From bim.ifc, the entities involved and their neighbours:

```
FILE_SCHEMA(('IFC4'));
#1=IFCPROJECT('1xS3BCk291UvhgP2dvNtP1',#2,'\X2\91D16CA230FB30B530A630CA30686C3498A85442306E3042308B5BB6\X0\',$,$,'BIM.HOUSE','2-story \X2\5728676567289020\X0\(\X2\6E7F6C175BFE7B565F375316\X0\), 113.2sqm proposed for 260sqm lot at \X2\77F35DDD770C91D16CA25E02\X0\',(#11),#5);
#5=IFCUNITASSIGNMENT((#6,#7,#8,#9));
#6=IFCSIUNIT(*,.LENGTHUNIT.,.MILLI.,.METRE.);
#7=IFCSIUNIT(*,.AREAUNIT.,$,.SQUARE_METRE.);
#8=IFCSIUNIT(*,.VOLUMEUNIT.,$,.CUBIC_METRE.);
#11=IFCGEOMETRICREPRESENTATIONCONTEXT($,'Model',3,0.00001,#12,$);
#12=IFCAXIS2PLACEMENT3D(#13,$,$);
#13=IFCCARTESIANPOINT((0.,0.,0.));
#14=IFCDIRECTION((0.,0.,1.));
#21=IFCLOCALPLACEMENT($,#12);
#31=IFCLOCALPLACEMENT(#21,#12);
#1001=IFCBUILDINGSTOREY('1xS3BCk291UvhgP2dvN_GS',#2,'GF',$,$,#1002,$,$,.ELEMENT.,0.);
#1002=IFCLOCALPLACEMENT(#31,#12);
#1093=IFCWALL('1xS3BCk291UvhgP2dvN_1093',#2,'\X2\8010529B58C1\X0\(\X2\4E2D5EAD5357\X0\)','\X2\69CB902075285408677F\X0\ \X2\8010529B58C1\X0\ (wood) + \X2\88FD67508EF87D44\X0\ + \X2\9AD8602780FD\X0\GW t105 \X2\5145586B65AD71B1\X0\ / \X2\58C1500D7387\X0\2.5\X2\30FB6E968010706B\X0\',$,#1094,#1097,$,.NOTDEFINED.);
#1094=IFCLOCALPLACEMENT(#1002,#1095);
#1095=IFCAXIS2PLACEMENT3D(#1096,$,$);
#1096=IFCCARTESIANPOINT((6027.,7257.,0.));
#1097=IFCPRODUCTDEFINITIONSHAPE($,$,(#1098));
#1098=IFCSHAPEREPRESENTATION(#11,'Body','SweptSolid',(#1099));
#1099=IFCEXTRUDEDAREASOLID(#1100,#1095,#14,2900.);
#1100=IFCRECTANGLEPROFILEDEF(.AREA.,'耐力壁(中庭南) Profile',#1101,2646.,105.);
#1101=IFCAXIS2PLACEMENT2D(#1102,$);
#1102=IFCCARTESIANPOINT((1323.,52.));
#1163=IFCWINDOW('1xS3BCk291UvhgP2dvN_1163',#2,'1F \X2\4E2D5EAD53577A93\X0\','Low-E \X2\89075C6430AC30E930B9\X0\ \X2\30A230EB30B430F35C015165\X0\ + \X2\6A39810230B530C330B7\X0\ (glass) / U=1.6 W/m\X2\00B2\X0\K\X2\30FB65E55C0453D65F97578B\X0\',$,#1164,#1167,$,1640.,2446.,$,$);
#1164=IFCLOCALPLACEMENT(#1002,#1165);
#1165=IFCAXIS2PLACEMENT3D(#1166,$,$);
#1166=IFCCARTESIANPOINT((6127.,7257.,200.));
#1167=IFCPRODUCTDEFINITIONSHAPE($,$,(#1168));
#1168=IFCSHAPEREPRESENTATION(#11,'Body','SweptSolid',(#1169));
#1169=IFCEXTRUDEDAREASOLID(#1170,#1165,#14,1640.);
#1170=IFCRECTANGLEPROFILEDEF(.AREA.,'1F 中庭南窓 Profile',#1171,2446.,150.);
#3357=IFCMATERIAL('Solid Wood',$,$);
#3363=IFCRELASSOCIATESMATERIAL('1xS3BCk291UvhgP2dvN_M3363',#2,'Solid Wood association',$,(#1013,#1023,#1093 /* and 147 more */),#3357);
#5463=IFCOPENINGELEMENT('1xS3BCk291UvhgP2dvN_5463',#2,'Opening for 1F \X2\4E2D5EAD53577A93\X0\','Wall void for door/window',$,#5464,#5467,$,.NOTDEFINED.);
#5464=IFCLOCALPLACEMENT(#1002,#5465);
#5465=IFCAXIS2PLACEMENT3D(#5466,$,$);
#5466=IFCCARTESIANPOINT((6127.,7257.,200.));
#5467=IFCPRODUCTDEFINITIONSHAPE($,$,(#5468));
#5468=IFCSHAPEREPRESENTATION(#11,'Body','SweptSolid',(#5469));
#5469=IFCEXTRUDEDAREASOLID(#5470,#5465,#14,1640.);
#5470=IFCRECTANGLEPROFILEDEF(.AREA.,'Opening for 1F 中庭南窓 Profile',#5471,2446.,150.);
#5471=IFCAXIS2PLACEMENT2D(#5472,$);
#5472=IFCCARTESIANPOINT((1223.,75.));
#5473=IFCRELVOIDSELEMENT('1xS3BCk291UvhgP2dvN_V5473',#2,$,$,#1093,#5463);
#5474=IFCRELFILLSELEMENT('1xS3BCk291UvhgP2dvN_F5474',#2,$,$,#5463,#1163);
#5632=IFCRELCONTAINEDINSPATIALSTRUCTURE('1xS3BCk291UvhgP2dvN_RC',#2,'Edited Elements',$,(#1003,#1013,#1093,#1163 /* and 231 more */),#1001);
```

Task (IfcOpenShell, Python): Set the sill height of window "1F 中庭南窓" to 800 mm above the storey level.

```python
import numpy as np
import ifcopenshell
import ifcopenshell.api.geometry
import ifcopenshell.geom
import ifcopenshell.util.element
import ifcopenshell.util.placement
import ifcopenshell.util.shape
import ifcopenshell.util.unit

model = ifcopenshell.open("bim.ifc")
unit_scale = ifcopenshell.util.unit.calculate_unit_scale(model)

window = model.by_guid("1xS3BCk291UvhgP2dvN_1163")
opening = window.FillsVoids[0].RelatingOpeningElement
storey = ifcopenshell.util.element.get_container(window, ifc_class="IfcBuildingStorey")
level = ifcopenshell.util.placement.get_local_placement(storey.ObjectPlacement)[2, 3]

# The opening's origin need not be at the sill, so measure its lowest point.
shape = ifcopenshell.geom.create_shape(ifcopenshell.geom.settings(), opening)
bottom = ifcopenshell.util.shape.get_shape_bottom_elevation(shape, shape.geometry) / unit_scale
dz = level + 800.0 - bottom

shift = np.array([0.0, 0.0, dz])
# The window is not placed relative to its opening, so move both.
for product in (opening, window):
    matrix = ifcopenshell.util.placement.get_local_placement(product.ObjectPlacement)
    matrix[:3, 3] += shift
    ifcopenshell.api.geometry.edit_object_placement(model, product=product, matrix=matrix, is_si=False)

print(f"moved by {dz * unit_scale:+.3f} m")

model.write("bim_v2.ifc")
```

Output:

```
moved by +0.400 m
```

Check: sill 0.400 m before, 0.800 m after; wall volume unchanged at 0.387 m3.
